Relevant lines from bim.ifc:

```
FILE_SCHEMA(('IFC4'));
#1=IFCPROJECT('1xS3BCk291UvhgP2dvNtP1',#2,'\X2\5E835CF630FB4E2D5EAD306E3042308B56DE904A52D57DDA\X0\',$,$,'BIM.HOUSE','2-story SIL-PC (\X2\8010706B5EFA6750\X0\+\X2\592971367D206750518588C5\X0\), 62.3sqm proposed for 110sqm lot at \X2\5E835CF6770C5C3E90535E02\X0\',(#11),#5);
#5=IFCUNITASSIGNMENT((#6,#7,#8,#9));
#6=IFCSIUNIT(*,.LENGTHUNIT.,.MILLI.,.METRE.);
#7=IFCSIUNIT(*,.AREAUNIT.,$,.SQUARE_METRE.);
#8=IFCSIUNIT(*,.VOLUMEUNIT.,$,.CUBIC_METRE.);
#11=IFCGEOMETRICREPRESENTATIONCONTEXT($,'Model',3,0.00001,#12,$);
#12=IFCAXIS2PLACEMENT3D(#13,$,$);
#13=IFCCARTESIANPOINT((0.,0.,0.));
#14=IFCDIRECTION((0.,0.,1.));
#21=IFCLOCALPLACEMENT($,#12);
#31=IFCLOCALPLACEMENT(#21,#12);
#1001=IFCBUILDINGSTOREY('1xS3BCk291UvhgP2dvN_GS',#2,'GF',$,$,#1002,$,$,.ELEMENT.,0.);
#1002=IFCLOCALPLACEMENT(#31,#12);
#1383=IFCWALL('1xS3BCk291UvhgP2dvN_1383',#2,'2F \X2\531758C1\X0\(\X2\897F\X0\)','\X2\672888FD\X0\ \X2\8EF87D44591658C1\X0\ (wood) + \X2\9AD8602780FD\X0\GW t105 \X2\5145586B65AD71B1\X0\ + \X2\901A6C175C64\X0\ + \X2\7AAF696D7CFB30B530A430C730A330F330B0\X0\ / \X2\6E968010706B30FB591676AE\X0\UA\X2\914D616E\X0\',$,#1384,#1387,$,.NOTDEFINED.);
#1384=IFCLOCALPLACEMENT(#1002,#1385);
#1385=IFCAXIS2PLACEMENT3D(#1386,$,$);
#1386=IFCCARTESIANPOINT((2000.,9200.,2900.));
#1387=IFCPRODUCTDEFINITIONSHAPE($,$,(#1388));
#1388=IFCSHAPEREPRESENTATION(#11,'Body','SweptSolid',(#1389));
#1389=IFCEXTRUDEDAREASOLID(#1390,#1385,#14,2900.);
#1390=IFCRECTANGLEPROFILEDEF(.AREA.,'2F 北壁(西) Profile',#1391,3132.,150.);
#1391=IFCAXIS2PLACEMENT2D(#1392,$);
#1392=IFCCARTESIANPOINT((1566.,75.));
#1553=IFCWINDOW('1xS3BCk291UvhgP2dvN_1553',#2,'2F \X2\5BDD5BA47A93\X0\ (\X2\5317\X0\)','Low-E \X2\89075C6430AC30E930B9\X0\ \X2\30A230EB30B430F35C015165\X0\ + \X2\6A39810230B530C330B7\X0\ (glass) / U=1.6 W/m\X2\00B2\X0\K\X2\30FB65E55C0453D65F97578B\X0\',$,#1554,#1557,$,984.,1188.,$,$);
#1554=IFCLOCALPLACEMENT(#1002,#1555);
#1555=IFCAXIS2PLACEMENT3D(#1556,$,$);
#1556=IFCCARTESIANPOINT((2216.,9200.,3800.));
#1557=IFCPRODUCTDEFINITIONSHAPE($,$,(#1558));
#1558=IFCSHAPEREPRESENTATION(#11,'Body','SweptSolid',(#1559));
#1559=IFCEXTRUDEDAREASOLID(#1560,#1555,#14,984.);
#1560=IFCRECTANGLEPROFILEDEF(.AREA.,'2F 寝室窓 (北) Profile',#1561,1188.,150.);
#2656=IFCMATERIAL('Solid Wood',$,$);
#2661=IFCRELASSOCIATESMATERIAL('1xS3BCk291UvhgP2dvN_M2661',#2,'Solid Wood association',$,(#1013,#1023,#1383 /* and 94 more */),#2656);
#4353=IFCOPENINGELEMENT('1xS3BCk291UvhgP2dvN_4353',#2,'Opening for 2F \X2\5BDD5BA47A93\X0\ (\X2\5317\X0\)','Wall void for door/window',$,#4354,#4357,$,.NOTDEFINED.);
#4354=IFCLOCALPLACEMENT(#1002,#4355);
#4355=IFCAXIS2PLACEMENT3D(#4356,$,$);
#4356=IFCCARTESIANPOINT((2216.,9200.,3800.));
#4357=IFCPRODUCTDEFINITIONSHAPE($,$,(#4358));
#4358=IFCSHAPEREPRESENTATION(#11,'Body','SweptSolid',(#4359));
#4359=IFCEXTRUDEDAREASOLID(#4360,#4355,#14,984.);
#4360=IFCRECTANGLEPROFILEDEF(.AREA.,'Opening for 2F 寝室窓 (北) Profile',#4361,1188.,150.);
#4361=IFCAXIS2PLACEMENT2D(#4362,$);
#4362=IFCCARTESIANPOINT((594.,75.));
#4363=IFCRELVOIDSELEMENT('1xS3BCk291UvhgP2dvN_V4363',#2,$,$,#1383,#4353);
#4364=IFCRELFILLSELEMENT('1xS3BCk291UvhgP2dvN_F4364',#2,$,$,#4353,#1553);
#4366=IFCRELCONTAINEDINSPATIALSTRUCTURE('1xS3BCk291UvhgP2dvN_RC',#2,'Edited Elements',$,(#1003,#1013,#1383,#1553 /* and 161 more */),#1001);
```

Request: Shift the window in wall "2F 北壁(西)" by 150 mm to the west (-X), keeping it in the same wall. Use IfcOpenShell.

```python
import ifcopenshell
import ifcopenshell.api.geometry
import ifcopenshell.util.placement
import ifcopenshell.util.unit

model = ifcopenshell.open("bim.ifc")
unit_scale = ifcopenshell.util.unit.calculate_unit_scale(model)

window = model.by_id(1553)
opening = window.FillsVoids[0].RelatingOpeningElement
wall = opening.VoidsElements[0].RelatingBuildingElement

wall_matrix = ifcopenshell.util.placement.get_local_placement(wall.ObjectPlacement)
shift = wall_matrix[:3, 0] * -0.15 / unit_scale
before = ifcopenshell.util.placement.get_local_placement(window.ObjectPlacement)[:3, 3].copy()

# The window is not placed relative to its opening, so move both.
for product in (opening, window):
    matrix = ifcopenshell.util.placement.get_local_placement(product.ObjectPlacement)
    matrix[:3, 3] += shift
    ifcopenshell.api.geometry.edit_object_placement(model, product=product, matrix=matrix, is_si=False)

after = ifcopenshell.util.placement.get_local_placement(window.ObjectPlacement)[:3, 3]
print("window moved by", (after - before).round(3) + 0.0)

model.write("bim_v2.ifc")
```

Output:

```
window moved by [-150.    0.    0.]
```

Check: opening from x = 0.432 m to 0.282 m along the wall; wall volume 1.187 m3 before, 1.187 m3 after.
